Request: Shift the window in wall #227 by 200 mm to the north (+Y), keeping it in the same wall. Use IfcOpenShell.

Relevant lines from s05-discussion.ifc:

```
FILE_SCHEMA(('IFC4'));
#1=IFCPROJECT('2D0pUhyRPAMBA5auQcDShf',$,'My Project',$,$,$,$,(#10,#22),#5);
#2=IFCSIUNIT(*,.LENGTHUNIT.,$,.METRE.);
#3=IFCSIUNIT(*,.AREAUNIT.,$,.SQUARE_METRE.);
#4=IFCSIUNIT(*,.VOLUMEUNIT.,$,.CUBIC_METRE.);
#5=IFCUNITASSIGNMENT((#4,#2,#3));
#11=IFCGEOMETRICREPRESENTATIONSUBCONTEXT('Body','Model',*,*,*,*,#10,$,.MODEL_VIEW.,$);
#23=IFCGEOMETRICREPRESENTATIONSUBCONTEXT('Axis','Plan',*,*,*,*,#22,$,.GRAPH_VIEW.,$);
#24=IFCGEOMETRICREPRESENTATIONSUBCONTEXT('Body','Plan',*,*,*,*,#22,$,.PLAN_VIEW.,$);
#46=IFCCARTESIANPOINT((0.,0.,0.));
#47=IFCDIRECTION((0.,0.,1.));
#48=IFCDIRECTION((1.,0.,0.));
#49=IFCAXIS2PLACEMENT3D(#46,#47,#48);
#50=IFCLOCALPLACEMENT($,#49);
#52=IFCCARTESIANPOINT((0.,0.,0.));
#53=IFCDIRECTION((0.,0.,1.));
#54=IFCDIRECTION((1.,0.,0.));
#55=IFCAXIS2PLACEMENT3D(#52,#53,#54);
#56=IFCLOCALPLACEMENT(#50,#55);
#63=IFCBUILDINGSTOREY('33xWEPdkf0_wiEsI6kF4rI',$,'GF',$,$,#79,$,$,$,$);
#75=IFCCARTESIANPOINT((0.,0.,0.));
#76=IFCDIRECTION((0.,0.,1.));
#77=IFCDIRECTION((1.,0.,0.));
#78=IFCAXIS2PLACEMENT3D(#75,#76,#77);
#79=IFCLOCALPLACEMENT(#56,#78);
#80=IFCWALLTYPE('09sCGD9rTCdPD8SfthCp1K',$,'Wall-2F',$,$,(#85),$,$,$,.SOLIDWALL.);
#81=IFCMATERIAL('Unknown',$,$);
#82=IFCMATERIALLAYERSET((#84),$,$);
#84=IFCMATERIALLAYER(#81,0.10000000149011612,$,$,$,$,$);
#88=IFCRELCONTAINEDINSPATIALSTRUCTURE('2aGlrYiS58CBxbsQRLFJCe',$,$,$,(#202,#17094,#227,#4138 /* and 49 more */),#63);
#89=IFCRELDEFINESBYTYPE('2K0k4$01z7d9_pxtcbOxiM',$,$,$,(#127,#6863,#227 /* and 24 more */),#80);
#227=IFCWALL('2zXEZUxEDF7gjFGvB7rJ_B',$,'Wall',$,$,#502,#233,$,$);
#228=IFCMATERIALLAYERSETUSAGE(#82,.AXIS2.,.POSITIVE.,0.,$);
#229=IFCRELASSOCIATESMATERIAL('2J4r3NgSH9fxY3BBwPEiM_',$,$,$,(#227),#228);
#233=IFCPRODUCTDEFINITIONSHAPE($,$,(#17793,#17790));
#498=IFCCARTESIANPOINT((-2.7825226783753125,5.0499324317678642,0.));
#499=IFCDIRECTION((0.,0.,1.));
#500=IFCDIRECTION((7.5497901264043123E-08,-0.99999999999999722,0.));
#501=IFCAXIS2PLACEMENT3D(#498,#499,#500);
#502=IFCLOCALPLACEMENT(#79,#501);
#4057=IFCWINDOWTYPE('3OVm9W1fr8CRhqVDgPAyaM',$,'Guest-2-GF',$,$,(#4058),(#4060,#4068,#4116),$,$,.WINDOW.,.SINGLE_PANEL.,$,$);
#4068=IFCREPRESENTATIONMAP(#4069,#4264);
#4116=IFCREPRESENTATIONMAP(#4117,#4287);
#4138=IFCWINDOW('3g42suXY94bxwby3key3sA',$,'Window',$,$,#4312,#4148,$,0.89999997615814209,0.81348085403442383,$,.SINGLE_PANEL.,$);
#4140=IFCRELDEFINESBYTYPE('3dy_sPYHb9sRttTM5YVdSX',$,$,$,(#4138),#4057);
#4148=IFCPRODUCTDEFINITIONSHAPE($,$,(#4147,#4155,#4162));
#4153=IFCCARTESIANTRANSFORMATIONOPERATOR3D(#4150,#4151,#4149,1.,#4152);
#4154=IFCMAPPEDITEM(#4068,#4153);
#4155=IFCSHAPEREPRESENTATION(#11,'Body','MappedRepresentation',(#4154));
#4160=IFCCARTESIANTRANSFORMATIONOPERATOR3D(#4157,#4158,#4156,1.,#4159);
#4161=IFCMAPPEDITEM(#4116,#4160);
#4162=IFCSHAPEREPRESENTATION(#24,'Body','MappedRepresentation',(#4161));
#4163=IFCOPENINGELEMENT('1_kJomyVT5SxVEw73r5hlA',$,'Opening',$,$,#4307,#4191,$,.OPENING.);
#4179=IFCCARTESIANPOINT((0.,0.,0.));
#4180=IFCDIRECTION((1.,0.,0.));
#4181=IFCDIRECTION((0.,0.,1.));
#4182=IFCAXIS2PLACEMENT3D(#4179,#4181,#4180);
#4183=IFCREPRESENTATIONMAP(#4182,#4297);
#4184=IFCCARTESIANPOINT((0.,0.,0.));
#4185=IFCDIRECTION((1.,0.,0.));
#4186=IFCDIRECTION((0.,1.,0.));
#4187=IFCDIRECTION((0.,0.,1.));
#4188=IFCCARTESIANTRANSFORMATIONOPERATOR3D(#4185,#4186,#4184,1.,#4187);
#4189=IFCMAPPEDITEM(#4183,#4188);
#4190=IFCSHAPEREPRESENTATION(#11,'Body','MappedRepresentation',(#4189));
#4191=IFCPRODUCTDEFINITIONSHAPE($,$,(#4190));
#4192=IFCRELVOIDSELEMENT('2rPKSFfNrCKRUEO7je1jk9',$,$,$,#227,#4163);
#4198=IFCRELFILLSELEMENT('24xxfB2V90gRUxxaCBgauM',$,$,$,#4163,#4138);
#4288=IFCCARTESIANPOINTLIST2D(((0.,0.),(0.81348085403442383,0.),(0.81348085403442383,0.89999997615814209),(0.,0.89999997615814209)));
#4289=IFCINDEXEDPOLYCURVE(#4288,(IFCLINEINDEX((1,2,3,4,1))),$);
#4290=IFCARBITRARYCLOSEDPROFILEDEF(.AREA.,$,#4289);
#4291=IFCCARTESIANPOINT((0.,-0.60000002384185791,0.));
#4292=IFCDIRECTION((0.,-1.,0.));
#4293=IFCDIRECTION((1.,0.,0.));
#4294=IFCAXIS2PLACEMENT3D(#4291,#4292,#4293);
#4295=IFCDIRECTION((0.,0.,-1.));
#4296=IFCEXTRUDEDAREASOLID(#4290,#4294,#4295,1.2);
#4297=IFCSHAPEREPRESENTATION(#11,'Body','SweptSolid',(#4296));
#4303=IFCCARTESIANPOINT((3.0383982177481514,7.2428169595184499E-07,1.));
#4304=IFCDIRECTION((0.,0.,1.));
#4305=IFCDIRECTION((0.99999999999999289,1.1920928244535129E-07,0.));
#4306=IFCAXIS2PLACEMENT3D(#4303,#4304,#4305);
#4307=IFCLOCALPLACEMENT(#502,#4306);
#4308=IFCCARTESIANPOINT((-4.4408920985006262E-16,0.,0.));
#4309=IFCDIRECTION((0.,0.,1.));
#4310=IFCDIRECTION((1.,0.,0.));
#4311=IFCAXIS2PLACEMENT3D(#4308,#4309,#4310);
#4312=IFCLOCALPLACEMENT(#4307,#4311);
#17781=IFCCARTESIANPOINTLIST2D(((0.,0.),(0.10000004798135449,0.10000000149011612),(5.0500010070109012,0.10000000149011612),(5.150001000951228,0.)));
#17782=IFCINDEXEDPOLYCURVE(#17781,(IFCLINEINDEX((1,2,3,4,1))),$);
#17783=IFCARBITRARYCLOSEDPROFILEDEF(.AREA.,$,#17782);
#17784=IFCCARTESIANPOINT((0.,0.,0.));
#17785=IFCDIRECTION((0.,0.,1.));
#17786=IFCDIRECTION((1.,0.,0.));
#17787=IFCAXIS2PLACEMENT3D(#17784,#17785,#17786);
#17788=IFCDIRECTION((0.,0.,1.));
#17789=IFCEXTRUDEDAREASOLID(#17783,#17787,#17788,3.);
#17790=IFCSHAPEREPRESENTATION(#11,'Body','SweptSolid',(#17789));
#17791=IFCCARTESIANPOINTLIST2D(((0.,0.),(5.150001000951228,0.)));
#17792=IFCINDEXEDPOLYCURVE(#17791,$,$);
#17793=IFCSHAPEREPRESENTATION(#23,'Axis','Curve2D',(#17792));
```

```python
import ifcopenshell
import ifcopenshell.api.geometry
import ifcopenshell.util.placement

model = ifcopenshell.open("s05-discussion.ifc")

window = model.by_id(4138)
opening = window.FillsVoids[0].RelatingOpeningElement
wall = opening.VoidsElements[0].RelatingBuildingElement

wall_matrix = ifcopenshell.util.placement.get_local_placement(wall.ObjectPlacement)
shift = wall_matrix[:3, 0] * -0.2
before = ifcopenshell.util.placement.get_local_placement(window.ObjectPlacement)[:3, 3].copy()

# The window is placed relative to its opening, so it follows when the opening moves.
matrix = ifcopenshell.util.placement.get_local_placement(opening.ObjectPlacement)
matrix[:3, 3] += shift
ifcopenshell.api.geometry.edit_object_placement(
    model, product=opening, matrix=matrix, is_si=False, should_transform_children=True
)

after = ifcopenshell.util.placement.get_local_placement(window.ObjectPlacement)[:3, 3]
print("window moved by", (after - before).round(3) + 0.0)

model.write("s05-discussion-out.ifc")
```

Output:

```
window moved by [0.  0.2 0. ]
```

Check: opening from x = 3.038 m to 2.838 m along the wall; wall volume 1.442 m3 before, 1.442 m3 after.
